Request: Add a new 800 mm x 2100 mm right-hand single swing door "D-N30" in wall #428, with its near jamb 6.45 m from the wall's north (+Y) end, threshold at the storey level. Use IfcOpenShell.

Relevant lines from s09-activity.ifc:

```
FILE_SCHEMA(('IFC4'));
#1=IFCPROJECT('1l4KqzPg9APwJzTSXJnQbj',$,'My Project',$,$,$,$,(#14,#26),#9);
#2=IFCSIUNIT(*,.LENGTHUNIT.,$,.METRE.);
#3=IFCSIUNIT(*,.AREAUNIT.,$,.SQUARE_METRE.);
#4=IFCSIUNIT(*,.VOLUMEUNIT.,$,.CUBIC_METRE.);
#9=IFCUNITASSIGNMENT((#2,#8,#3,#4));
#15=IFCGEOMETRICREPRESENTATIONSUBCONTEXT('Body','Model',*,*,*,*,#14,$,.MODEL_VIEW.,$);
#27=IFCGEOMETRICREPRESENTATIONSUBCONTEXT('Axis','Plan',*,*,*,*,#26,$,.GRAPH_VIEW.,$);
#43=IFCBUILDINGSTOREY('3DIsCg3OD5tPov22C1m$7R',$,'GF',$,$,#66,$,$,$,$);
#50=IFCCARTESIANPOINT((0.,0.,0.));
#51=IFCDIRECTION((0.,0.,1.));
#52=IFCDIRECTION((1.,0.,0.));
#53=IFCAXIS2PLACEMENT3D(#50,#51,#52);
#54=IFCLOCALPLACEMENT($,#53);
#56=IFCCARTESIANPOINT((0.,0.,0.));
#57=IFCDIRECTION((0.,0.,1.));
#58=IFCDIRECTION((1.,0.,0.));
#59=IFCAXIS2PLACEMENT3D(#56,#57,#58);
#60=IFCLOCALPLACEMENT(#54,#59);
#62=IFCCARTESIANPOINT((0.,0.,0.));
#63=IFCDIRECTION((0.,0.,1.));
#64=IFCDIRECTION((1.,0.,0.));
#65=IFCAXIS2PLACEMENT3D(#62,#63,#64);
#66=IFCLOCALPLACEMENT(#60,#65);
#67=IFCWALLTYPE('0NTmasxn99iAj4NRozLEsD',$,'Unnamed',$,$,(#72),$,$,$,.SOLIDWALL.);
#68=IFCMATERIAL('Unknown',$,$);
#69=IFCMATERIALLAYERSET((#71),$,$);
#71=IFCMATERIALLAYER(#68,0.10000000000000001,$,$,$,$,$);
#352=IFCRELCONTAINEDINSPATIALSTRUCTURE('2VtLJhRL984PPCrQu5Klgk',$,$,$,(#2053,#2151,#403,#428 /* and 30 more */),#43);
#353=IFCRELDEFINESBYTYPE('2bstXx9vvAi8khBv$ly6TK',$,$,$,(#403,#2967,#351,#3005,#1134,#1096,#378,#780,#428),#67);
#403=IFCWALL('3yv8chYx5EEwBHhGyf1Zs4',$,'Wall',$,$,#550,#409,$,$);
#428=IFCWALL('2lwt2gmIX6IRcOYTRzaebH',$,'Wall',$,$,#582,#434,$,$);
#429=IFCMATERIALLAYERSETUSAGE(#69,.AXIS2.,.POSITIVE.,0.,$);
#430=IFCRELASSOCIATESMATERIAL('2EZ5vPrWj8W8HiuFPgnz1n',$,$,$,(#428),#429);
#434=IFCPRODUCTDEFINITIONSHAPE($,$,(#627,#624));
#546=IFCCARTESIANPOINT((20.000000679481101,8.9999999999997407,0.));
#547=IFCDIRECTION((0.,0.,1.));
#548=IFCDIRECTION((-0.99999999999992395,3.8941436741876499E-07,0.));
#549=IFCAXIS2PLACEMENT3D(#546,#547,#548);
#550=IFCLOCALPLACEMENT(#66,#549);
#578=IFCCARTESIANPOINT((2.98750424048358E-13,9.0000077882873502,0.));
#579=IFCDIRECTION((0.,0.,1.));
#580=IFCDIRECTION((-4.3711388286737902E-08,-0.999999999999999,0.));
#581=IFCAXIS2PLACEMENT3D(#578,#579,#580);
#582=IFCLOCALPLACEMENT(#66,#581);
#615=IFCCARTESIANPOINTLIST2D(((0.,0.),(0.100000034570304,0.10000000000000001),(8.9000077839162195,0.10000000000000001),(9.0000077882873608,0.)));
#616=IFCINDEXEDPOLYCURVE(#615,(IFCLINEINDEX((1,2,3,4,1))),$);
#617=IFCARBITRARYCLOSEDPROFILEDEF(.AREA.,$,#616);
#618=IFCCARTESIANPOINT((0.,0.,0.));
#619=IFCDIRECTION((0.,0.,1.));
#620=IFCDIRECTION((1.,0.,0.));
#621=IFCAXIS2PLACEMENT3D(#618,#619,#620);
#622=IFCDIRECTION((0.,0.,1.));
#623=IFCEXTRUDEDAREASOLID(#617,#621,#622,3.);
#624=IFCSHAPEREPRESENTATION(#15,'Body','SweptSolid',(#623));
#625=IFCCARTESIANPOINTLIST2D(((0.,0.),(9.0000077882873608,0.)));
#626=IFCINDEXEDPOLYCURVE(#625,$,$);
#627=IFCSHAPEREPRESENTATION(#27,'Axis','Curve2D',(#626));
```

```python
import numpy as np
import ifcopenshell
import ifcopenshell.api.feature
import ifcopenshell.api.geometry
import ifcopenshell.api.root
import ifcopenshell.api.spatial
import ifcopenshell.geom
import ifcopenshell.util.element
import ifcopenshell.util.placement
import ifcopenshell.util.representation
import ifcopenshell.util.shape
import ifcopenshell.util.unit

model = ifcopenshell.open("s09-activity.ifc")
unit_scale = ifcopenshell.util.unit.calculate_unit_scale(model)
settings = ifcopenshell.geom.settings()


def volume(element):
    """Net volume in cubic metres, openings subtracted."""
    shape = ifcopenshell.geom.create_shape(settings, element)
    return ifcopenshell.util.shape.get_volume(shape.geometry)


wall = model.by_id(428)
storey = ifcopenshell.util.element.get_container(wall, ifc_class="IfcBuildingStorey")
context = ifcopenshell.util.representation.get_context(model, "Model", "Body", "MODEL_VIEW")
before = volume(wall)

width, height, from_end, sill = 0.8, 2.1, 6.45, 0.0  # metres

# The wall runs along its own X axis, and the end named is its -X end.
wall_shape = ifcopenshell.geom.create_shape(settings, wall)
x, y, z = ifcopenshell.util.shape.get_vertices(wall_shape.geometry).T
start = x.min() + from_end
face, thickness = float(y.min()), float(y.max() - y.min())
wall_matrix = ifcopenshell.util.placement.get_local_placement(wall.ObjectPlacement)
level = ifcopenshell.util.placement.get_local_placement(storey.ObjectPlacement)[2, 3]


def in_wall(x, y):
    """Placement at x, y metres in the wall's axes, at sill height."""
    matrix = wall_matrix.copy()
    matrix[:, 3] = wall_matrix @ np.array([x / unit_scale, y / unit_scale, 0.0, 1.0])
    matrix[2, 3] = level + sill / unit_scale
    return matrix


# Opening: a box that overshoots both wall faces by 50 mm.
opening = ifcopenshell.api.root.create_entity(model, ifc_class="IfcOpeningElement", predefined_type="OPENING")
box = ifcopenshell.api.geometry.add_wall_representation(
    model, context=context, length=width, height=height, thickness=thickness + 0.1
)
ifcopenshell.api.geometry.assign_representation(model, product=opening, representation=box)
ifcopenshell.api.geometry.edit_object_placement(model, product=opening, matrix=in_wall(start, face - 0.05), is_si=False)
ifcopenshell.api.feature.add_feature(model, feature=opening, element=wall)

door = ifcopenshell.api.root.create_entity(model, ifc_class="IfcDoor", name="D-N30", predefined_type="DOOR")
door.OverallWidth, door.OverallHeight = width / unit_scale, height / unit_scale
door.OperationType = "SINGLE_SWING_RIGHT"
body = ifcopenshell.api.geometry.add_door_representation(
    model,
    context=context,
    overall_width=door.OverallWidth,
    overall_height=door.OverallHeight,
    operation_type="SINGLE_SWING_RIGHT",
    lining_properties={"LiningDepth": thickness / unit_scale, "ThresholdDepth": thickness / unit_scale},
)
ifcopenshell.api.geometry.assign_representation(model, product=door, representation=body)
ifcopenshell.api.spatial.assign_container(model, products=[door], relating_structure=storey)
ifcopenshell.api.feature.add_filling(model, opening=opening, element=door)

# The lining spans the wall, so the door starts at the wall face.
ifcopenshell.api.geometry.edit_object_placement(model, product=door, matrix=in_wall(start, face), is_si=False)

after = volume(wall)

print(f"wall volume {before:.3f} -> {after:.3f} m3")

model.write("s09-activity-out.ifc")
```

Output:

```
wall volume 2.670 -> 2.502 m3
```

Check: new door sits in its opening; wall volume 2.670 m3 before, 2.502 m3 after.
